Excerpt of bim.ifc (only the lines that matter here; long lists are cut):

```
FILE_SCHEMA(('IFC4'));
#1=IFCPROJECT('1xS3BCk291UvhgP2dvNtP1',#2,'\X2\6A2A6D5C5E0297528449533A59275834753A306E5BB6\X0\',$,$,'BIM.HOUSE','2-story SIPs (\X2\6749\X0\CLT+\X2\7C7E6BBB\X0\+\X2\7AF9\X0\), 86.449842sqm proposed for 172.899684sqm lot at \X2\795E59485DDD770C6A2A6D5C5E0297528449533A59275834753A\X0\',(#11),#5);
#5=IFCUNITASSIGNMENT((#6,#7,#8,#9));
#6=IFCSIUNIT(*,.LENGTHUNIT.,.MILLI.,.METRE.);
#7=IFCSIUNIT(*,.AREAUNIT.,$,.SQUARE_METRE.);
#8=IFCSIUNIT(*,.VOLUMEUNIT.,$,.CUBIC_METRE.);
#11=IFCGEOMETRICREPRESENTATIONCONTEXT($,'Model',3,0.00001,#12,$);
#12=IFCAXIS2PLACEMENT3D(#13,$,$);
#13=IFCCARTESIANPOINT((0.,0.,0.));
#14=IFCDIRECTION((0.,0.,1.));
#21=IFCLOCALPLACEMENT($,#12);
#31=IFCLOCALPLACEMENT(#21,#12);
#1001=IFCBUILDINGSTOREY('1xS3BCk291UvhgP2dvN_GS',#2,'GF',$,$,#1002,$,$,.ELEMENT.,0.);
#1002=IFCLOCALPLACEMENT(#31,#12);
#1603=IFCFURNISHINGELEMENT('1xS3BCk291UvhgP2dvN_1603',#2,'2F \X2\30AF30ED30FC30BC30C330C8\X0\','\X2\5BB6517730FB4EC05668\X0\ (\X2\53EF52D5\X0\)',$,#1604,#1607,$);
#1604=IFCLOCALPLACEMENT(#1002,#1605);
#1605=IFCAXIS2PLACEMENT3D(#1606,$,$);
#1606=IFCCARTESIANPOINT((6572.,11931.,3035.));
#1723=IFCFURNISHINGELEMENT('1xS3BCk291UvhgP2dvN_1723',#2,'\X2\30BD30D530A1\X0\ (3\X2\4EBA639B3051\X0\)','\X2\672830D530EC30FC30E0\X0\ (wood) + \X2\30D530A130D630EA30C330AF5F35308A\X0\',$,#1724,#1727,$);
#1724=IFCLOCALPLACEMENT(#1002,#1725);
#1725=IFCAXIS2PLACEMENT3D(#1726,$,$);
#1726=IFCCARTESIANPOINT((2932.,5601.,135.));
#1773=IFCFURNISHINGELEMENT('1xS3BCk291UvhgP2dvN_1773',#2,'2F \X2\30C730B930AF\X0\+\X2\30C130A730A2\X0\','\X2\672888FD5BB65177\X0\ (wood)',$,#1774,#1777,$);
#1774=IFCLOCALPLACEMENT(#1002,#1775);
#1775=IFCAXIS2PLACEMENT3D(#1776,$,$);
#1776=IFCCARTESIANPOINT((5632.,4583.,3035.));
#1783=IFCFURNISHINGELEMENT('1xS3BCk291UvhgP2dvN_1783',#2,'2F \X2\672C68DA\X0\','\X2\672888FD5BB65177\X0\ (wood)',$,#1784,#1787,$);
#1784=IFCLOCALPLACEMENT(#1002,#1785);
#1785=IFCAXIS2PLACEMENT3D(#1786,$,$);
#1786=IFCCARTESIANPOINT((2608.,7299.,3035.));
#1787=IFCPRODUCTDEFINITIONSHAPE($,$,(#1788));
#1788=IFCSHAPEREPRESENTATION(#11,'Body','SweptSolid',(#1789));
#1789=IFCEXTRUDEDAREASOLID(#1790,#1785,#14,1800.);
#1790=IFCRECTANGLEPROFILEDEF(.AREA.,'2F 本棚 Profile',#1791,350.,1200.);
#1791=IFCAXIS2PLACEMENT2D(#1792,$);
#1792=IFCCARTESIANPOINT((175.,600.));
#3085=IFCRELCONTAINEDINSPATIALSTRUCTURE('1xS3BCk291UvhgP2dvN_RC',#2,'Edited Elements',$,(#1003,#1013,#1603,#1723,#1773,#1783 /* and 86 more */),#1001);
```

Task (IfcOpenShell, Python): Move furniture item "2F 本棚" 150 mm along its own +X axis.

```python
import ifcopenshell
import ifcopenshell.api.geometry
import ifcopenshell.util.placement

model = ifcopenshell.open("bim.ifc")

item = model.by_id(1783)
matrix = ifcopenshell.util.placement.get_local_placement(item.ObjectPlacement)
matrix[:3, 3] += matrix[:3, 0] * 150.0
ifcopenshell.api.geometry.edit_object_placement(model, product=item, matrix=matrix, is_si=False)

print(ifcopenshell.util.placement.get_local_placement(item.ObjectPlacement).round(3) + 0.0)

model.write("bim_edited.ifc")
```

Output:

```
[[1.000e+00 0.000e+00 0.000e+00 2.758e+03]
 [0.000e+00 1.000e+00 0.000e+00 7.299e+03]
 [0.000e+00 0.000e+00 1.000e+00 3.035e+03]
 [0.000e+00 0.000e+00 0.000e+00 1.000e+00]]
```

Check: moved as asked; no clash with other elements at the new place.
